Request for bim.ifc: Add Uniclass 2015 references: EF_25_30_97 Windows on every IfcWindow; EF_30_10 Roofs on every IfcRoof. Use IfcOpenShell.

First a look at what the model holds.

```python
import ifcopenshell

model = ifcopenshell.open("bim.ifc")
print(model.schema)
print("classifications:", [c.Name for c in model.by_type("IfcClassification")])
for ifc_class in ("IfcDoor", "IfcRoof", "IfcStair", "IfcWall", "IfcWindow"):
    print(ifc_class, len(model.by_type(ifc_class)))
```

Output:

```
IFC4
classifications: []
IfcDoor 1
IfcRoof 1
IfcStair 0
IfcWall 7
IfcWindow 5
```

```python
import ifcopenshell
import ifcopenshell.api.classification

model = ifcopenshell.open("bim.ifc")

system = ifcopenshell.api.classification.add_classification(model, classification="Uniclass 2015")

codes = {
    "IfcWindow": ("EF_25_30_97", "Windows"),
    "IfcRoof": ("EF_30_10", "Roofs"),
}
for ifc_class, (code, name) in codes.items():
    products = model.by_type(ifc_class)
    ifcopenshell.api.classification.add_reference(
        model, products=products, classification=system, identification=code, name=name
    )
    print(code, len(products))

model.write("bim-out.ifc")
```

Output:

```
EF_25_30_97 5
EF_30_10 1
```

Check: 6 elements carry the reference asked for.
